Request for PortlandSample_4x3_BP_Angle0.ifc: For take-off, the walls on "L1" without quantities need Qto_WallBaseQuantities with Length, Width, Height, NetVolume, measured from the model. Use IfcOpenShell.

First a look at what the model holds.

```python
import ifcopenshell
import ifcopenshell.util.element
import ifcopenshell.util.unit

model = ifcopenshell.open("PortlandSample_4x3_BP_Angle0.ifc")
print(model.schema)
for unit_type in ("LENGTHUNIT", "AREAUNIT", "VOLUMEUNIT"):
    print(unit_type, ifcopenshell.util.unit.calculate_unit_scale(model, unit_type))
storey = next(s for s in model.by_type("IfcBuildingStorey") if s.Name == "L1")
walls = [e for e in ifcopenshell.util.element.get_decomposition(storey) if e.is_a("IfcWall")]
for e in sorted(walls, key=lambda e: e.id()):
    print(e.id(), e.is_a(), e.Name, list(ifcopenshell.util.element.get_psets(e, qtos_only=True)), sep=" | ")
```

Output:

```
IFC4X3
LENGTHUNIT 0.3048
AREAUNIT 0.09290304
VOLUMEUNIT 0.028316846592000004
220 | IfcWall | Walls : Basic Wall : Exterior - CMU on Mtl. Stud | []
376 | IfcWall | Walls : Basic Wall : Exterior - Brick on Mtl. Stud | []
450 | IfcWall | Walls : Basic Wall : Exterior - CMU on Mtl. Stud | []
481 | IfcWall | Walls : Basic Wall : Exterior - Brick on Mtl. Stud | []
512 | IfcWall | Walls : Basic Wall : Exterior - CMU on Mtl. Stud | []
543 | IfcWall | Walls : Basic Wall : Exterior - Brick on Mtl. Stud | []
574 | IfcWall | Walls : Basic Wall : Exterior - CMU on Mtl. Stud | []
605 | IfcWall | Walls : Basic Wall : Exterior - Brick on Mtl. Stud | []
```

```python
import ifcopenshell
import ifcopenshell.api.pset
import ifcopenshell.geom
import ifcopenshell.util.element
import ifcopenshell.util.shape
import ifcopenshell.util.unit

model = ifcopenshell.open("PortlandSample_4x3_BP_Angle0.ifc")
unit_scale = ifcopenshell.util.unit.calculate_unit_scale(model)
volume_scale = ifcopenshell.util.unit.calculate_unit_scale(model, "VOLUMEUNIT")
settings = ifcopenshell.geom.settings()

storey = next(s for s in model.by_type("IfcBuildingStorey") if s.Name == "L1")
walls = [e for e in ifcopenshell.util.element.get_decomposition(storey) if e.is_a("IfcWall")]

for e in sorted(walls, key=lambda e: e.id()):
    if ifcopenshell.util.element.get_psets(e, qtos_only=True, should_inherit=False):
        continue
    # Geometry comes back in metres, in the element's own axes.
    shape = ifcopenshell.geom.create_shape(settings, e)
    values = {
        "Length": ifcopenshell.util.shape.get_x(shape.geometry) / unit_scale,
        "Width": ifcopenshell.util.shape.get_y(shape.geometry) / unit_scale,
        "Height": ifcopenshell.util.shape.get_z(shape.geometry) / unit_scale,
        "NetVolume": ifcopenshell.util.shape.get_volume(shape.geometry) / volume_scale,
    }
    qto = ifcopenshell.api.pset.add_qto(model, product=e, name="Qto_WallBaseQuantities")
    ifcopenshell.api.pset.edit_qto(model, qto=qto, properties=values)
    print(e.id(), {k: round(v, 3) for k, v in values.items()})

model.write("PortlandSample_4x3_BP_Angle0_updated.ifc")
```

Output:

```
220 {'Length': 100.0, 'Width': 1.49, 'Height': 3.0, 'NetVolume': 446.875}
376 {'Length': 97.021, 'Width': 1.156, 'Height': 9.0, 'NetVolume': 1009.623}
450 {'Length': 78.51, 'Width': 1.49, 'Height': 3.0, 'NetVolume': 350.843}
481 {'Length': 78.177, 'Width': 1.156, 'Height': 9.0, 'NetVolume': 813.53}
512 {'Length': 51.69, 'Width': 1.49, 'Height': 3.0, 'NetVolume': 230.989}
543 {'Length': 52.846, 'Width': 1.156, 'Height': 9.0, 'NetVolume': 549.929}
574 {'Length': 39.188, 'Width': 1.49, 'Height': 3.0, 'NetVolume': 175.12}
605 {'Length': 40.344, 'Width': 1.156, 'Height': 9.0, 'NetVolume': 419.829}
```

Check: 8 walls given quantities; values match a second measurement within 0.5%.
